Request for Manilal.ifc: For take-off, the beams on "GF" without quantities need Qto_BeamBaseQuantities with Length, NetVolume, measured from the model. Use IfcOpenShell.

First a look at what the model holds.

```python
import ifcopenshell
import ifcopenshell.util.element
import ifcopenshell.util.unit

model = ifcopenshell.open("Manilal.ifc")
print(model.schema)
for unit_type in ("LENGTHUNIT", "AREAUNIT", "VOLUMEUNIT"):
    print(unit_type, ifcopenshell.util.unit.calculate_unit_scale(model, unit_type))
storey = next(s for s in model.by_type("IfcBuildingStorey") if s.Name == "GF")
beams = [e for e in ifcopenshell.util.element.get_decomposition(storey) if e.is_a("IfcBeam")]
for e in sorted(beams, key=lambda e: e.id()):
    print(e.id(), e.is_a(), e.Name, list(ifcopenshell.util.element.get_psets(e, qtos_only=True)), sep=" | ")
```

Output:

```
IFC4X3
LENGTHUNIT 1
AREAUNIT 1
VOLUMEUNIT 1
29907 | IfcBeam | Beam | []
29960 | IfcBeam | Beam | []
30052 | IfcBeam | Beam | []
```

```python
import ifcopenshell
import ifcopenshell.api.pset
import ifcopenshell.geom
import ifcopenshell.util.element
import ifcopenshell.util.shape
import ifcopenshell.util.unit

model = ifcopenshell.open("Manilal.ifc")
unit_scale = ifcopenshell.util.unit.calculate_unit_scale(model)
volume_scale = ifcopenshell.util.unit.calculate_unit_scale(model, "VOLUMEUNIT")
settings = ifcopenshell.geom.settings()

storey = next(s for s in model.by_type("IfcBuildingStorey") if s.Name == "GF")
beams = [e for e in ifcopenshell.util.element.get_decomposition(storey) if e.is_a("IfcBeam")]

for e in sorted(beams, key=lambda e: e.id()):
    if ifcopenshell.util.element.get_psets(e, qtos_only=True, should_inherit=False):
        continue
    # Geometry comes back in metres, in the element's own axes.
    shape = ifcopenshell.geom.create_shape(settings, e)
    values = {
        "Length": ifcopenshell.util.shape.get_max_xyz(shape.geometry) / unit_scale,
        "NetVolume": ifcopenshell.util.shape.get_volume(shape.geometry) / volume_scale,
    }
    qto = ifcopenshell.api.pset.add_qto(model, product=e, name="Qto_BeamBaseQuantities")
    ifcopenshell.api.pset.edit_qto(model, qto=qto, properties=values)
    print(e.id(), {k: round(v, 3) for k, v in values.items()})

model.write("Manilal-out.ifc")
```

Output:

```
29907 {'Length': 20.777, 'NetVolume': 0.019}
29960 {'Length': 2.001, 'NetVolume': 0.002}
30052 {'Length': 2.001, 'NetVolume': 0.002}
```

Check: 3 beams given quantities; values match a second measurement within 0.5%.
